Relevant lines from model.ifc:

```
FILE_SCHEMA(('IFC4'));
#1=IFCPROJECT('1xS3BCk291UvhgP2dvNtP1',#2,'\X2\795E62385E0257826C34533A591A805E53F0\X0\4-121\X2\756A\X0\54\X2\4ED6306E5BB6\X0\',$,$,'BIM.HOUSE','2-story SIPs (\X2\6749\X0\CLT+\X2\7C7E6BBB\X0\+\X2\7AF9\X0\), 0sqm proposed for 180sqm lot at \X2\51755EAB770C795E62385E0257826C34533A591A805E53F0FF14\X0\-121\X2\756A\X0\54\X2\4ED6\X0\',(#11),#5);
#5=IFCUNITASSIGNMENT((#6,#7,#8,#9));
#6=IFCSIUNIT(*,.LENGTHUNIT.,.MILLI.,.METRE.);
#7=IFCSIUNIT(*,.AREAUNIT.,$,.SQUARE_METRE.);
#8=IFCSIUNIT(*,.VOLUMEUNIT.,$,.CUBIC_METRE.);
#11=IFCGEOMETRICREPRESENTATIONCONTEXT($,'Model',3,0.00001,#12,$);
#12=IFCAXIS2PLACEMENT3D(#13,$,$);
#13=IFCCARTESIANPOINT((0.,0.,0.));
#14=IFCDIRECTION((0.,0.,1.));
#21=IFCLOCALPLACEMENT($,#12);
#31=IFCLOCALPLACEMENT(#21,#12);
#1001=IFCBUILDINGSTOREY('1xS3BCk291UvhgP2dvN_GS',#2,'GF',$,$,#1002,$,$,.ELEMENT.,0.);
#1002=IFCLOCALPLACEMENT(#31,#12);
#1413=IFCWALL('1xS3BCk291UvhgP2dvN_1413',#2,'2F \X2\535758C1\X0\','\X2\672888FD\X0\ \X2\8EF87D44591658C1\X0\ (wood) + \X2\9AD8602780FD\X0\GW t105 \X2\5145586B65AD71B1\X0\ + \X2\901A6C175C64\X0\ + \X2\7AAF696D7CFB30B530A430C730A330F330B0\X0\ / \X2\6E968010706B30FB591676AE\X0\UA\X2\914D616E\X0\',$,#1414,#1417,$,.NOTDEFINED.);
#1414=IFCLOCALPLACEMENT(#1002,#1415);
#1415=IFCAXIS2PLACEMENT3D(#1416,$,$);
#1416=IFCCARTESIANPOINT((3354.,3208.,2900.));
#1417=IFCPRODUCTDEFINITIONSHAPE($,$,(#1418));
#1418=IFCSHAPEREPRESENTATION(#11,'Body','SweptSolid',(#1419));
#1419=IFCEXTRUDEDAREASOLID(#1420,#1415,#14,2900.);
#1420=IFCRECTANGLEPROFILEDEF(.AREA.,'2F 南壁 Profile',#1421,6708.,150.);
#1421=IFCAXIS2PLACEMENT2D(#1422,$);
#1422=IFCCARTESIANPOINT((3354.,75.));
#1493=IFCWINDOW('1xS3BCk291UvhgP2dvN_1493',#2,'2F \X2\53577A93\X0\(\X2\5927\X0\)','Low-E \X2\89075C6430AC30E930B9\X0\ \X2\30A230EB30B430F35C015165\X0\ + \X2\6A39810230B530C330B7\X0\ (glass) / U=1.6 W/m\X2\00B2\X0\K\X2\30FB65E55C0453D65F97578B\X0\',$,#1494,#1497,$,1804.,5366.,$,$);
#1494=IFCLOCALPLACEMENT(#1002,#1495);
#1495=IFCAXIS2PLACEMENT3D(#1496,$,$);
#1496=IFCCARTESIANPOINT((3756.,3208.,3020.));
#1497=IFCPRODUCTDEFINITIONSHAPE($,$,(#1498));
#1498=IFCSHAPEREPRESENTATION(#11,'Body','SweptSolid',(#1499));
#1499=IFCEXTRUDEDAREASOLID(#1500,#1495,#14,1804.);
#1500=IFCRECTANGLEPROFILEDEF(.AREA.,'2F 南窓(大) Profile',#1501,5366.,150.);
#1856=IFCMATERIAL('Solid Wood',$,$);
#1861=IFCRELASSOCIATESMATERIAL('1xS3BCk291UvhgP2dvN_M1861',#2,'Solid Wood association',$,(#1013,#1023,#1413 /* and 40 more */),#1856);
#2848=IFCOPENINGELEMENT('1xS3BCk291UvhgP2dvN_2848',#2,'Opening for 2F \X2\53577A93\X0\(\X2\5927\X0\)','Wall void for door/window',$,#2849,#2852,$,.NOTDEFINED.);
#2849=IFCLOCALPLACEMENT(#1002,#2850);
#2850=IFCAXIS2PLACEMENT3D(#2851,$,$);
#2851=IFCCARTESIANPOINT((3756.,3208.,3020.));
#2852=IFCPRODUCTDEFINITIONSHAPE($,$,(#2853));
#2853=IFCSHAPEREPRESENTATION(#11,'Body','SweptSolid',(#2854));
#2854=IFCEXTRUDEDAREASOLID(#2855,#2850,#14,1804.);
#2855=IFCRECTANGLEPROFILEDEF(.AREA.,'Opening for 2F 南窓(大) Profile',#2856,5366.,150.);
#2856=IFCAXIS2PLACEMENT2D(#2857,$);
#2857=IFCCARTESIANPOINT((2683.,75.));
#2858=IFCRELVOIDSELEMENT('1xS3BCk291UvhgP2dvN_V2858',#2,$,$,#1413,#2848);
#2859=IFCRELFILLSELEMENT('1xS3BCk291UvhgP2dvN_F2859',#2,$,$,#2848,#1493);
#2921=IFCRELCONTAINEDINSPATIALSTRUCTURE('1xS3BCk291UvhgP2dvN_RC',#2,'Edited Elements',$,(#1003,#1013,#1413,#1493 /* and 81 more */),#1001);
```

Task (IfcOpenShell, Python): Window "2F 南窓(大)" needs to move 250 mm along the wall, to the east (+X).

```python
import ifcopenshell
import ifcopenshell.api.geometry
import ifcopenshell.util.placement
import ifcopenshell.util.unit

model = ifcopenshell.open("model.ifc")
unit_scale = ifcopenshell.util.unit.calculate_unit_scale(model)

window = model.by_id(1493)
opening = window.FillsVoids[0].RelatingOpeningElement
wall = opening.VoidsElements[0].RelatingBuildingElement

wall_matrix = ifcopenshell.util.placement.get_local_placement(wall.ObjectPlacement)
shift = wall_matrix[:3, 0] * 0.25 / unit_scale
before = ifcopenshell.util.placement.get_local_placement(window.ObjectPlacement)[:3, 3].copy()

# The window is not placed relative to its opening, so move both.
for product in (opening, window):
    matrix = ifcopenshell.util.placement.get_local_placement(product.ObjectPlacement)
    matrix[:3, 3] += shift
    ifcopenshell.api.geometry.edit_object_placement(model, product=product, matrix=matrix, is_si=False)

after = ifcopenshell.util.placement.get_local_placement(window.ObjectPlacement)[:3, 3]
print("window moved by", (after - before).round(3) + 0.0)

model.write("model-out.ifc")
```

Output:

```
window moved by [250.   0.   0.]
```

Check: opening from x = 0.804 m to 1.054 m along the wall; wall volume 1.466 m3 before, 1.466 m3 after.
